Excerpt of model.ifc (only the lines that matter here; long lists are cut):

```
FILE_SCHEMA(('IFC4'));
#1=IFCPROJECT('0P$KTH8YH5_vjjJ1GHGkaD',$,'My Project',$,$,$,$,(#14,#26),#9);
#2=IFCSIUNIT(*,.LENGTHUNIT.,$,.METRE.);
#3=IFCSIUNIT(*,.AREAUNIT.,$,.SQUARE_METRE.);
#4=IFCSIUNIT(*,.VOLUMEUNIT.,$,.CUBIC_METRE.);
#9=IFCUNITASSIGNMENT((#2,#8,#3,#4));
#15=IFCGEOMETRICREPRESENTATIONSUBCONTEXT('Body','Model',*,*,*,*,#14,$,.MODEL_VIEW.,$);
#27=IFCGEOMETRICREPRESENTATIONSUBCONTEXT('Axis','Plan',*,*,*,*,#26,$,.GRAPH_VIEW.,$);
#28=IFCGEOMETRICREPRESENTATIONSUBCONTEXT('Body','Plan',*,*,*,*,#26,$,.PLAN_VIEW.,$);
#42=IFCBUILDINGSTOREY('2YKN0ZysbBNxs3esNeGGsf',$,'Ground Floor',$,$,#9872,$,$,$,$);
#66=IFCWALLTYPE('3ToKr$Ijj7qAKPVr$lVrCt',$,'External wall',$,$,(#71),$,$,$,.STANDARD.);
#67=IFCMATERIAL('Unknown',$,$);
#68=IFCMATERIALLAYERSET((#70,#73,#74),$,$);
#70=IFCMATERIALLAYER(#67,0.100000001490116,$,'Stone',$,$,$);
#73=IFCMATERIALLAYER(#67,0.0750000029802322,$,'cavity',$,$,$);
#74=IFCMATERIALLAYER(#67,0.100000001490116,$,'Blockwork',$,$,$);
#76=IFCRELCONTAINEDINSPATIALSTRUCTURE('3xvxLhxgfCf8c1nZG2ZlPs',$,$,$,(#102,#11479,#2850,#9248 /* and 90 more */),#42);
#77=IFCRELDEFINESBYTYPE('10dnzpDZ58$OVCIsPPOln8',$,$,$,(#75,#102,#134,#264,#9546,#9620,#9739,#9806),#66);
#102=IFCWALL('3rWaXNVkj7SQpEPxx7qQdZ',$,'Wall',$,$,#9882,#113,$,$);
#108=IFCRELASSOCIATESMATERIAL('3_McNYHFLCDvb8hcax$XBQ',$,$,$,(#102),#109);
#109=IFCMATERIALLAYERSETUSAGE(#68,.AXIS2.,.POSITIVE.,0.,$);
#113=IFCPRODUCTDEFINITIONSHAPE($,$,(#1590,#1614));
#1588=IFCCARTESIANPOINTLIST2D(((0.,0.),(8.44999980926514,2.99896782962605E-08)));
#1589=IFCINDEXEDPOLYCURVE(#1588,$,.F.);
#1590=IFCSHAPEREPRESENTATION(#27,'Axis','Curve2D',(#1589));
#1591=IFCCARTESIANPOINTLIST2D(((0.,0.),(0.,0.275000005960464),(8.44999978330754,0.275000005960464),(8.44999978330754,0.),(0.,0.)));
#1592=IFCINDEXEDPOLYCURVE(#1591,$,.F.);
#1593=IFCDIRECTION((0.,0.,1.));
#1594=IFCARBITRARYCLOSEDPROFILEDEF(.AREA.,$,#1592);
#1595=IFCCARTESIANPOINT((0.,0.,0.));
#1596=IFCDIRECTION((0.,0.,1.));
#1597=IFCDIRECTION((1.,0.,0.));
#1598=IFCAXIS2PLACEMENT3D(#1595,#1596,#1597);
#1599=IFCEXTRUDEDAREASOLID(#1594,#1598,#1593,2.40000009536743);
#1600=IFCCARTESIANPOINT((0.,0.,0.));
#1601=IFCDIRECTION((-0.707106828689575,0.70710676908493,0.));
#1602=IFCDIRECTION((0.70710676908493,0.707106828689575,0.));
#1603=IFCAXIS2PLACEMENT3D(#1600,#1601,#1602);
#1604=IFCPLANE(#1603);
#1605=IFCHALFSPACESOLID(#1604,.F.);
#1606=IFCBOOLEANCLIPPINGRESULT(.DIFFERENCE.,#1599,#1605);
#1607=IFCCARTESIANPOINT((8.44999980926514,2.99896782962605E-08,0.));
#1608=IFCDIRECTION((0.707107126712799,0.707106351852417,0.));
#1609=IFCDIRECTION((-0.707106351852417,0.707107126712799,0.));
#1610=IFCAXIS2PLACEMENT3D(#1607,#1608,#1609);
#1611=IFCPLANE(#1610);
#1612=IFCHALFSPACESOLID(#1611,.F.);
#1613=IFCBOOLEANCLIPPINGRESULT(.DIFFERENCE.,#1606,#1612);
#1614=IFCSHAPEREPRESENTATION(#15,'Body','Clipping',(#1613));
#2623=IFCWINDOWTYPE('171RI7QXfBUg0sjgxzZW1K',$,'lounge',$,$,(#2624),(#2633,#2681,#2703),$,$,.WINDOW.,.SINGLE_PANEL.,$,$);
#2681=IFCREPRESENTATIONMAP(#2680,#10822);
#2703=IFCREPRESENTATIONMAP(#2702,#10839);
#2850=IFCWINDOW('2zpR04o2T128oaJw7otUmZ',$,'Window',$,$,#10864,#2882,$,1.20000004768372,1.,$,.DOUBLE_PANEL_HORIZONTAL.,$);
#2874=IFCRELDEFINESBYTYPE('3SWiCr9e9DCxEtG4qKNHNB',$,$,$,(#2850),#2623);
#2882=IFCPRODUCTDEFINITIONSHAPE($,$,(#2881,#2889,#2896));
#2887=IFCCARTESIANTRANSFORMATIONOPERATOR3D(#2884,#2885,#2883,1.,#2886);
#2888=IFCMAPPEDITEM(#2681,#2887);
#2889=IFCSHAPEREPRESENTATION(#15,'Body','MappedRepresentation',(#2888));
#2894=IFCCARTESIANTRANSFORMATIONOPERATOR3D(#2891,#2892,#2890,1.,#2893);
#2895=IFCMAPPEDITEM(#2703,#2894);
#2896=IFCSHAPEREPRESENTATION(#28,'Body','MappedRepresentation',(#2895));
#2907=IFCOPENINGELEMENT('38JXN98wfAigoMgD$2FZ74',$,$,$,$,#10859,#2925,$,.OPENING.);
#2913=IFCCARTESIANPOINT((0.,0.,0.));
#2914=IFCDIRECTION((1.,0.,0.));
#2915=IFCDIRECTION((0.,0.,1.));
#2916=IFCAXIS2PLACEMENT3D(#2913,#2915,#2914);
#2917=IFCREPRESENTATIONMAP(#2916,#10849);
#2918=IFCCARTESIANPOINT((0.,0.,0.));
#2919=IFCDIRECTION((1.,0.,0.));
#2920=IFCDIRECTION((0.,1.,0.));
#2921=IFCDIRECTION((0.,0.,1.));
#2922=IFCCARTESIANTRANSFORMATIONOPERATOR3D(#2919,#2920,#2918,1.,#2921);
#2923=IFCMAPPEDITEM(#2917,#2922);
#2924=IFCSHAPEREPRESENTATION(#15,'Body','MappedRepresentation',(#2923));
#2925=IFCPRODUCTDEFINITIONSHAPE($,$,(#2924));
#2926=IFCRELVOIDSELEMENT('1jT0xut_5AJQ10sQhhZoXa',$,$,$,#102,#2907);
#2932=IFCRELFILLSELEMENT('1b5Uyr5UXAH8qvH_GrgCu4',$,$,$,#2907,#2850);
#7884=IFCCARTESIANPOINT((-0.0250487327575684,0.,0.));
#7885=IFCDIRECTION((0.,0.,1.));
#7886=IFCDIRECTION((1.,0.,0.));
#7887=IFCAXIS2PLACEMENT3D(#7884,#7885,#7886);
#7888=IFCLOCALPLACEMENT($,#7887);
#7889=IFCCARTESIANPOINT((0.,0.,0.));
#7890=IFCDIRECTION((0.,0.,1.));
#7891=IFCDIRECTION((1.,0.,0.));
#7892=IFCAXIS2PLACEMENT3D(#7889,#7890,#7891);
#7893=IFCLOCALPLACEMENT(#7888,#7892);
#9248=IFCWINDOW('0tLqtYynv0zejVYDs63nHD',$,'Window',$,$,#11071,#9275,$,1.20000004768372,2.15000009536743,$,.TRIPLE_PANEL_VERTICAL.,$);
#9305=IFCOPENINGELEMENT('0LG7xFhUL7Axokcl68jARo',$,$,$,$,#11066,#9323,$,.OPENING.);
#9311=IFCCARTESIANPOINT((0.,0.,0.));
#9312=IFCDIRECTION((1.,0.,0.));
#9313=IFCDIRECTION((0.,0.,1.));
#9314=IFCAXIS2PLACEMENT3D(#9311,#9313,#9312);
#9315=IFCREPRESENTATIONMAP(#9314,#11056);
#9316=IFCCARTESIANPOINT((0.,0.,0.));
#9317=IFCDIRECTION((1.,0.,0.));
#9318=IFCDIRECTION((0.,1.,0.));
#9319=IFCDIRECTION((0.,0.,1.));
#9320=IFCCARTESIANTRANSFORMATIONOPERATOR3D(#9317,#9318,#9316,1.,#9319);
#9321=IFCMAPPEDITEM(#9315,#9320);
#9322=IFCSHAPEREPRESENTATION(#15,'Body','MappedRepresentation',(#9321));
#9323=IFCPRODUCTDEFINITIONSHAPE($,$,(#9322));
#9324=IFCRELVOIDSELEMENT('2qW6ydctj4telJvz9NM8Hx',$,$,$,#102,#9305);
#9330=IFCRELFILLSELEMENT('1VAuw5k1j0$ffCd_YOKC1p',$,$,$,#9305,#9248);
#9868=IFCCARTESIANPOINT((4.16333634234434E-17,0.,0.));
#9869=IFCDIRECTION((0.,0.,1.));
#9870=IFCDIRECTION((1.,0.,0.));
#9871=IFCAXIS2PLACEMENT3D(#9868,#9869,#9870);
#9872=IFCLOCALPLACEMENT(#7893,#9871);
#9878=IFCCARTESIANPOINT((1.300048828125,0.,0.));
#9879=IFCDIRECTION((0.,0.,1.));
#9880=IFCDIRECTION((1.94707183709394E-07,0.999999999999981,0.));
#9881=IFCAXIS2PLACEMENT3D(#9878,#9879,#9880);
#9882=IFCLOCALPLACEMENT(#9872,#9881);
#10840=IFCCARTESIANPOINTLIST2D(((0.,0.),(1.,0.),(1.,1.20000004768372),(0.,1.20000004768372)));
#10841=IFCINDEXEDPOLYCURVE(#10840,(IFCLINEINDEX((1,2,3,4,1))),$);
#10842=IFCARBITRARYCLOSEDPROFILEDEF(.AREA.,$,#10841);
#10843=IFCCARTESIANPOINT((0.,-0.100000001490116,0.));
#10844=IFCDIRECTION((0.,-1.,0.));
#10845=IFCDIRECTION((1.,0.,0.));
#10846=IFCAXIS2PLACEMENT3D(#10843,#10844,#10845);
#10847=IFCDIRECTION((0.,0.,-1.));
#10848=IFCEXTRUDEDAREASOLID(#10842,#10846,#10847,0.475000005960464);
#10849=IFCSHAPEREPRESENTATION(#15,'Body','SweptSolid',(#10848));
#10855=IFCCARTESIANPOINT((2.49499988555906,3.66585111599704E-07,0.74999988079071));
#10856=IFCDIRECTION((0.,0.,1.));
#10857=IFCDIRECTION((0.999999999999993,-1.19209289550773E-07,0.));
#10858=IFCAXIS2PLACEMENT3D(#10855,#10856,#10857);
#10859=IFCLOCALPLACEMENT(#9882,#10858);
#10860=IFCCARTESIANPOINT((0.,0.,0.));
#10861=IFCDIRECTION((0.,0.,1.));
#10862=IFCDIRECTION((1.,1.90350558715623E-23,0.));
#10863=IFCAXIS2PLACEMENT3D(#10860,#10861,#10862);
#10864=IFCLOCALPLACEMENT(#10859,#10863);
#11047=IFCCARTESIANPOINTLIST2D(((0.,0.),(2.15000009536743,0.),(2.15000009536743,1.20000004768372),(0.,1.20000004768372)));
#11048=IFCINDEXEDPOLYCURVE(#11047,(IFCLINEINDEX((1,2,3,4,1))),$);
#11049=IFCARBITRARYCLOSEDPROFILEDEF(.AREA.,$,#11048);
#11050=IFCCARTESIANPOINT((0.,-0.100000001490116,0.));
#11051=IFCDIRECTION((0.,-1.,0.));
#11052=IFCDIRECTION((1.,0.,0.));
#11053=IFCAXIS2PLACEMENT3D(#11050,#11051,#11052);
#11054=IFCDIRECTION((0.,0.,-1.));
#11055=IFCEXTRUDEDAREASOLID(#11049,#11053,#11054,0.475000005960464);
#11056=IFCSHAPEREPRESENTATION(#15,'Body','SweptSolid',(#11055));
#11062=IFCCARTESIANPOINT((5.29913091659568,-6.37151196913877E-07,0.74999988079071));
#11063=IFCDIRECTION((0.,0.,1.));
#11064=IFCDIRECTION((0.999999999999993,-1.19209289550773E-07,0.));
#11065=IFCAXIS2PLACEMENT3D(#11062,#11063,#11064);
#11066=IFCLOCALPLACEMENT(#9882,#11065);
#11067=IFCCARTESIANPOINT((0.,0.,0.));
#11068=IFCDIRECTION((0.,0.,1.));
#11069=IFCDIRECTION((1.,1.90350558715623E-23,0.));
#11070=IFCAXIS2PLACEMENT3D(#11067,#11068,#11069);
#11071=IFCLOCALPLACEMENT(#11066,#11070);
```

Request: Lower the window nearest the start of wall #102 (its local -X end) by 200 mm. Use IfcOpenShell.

```python
import numpy as np
import ifcopenshell
import ifcopenshell.api.geometry
import ifcopenshell.util.placement
import ifcopenshell.util.unit

model = ifcopenshell.open("model.ifc")
unit_scale = ifcopenshell.util.unit.calculate_unit_scale(model)

window = model.by_guid("2zpR04o2T128oaJw7otUmZ")
opening = window.FillsVoids[0].RelatingOpeningElement
dz = -0.2 / unit_scale

shift = np.array([0.0, 0.0, dz])
# The window is placed relative to its opening, so it follows when the opening moves.
matrix = ifcopenshell.util.placement.get_local_placement(opening.ObjectPlacement)
matrix[:3, 3] += shift
ifcopenshell.api.geometry.edit_object_placement(
    model, product=opening, matrix=matrix, is_si=False, should_transform_children=True
)

print(f"moved by {dz * unit_scale:+.3f} m")

model.write("model_edited.ifc")
```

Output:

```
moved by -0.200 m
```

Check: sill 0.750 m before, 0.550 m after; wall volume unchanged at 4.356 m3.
